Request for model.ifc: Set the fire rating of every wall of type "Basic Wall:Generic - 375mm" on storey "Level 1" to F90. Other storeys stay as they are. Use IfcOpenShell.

First a look at what the model holds.

```python
import ifcopenshell
import ifcopenshell.util.element

model = ifcopenshell.open("model.ifc")
print(model.schema)
storey = next(s for s in model.by_type("IfcBuildingStorey") if s.Name == "Level 1")
walls = [e for e in ifcopenshell.util.element.get_decomposition(storey) if e.is_a("IfcWall")]
seen = {}
for e in walls:
    element_type = ifcopenshell.util.element.get_type(e)
    key = (element_type.Name if element_type != e and element_type else None, ifcopenshell.util.element.get_pset(e, "Pset_WallCommon", "FireRating"))
    seen[key] = seen.get(key, 0) + 1
for (name, value), count in sorted(seen.items(), key=str):
    print(count, "x", name, "|", value)
```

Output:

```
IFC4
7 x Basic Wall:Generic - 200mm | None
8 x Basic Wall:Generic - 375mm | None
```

```python
import ifcopenshell
import ifcopenshell.api.pset
import ifcopenshell.util.element

model = ifcopenshell.open("model.ifc")

storey = next(s for s in model.by_type("IfcBuildingStorey") if s.Name == "Level 1")
walls = [e for e in ifcopenshell.util.element.get_decomposition(storey) if e.is_a("IfcWall")]

count = 0
for e in walls:
    element_type = ifcopenshell.util.element.get_type(e)
    if element_type in (None, e) or element_type.Name != "Basic Wall:Generic - 375mm":
        continue
    # add_pset returns the element's existing set when there is one.
    pset = ifcopenshell.api.pset.add_pset(model, product=e, name="Pset_WallCommon")
    ifcopenshell.api.pset.edit_pset(model, pset=pset, properties={"FireRating": "F90"})
    count += 1

print(count, "walls updated")

model.write("model_v2.ifc")
```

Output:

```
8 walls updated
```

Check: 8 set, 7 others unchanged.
